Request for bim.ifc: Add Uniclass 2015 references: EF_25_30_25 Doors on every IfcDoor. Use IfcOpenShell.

First a look at what the model holds.

```python
import ifcopenshell

model = ifcopenshell.open("bim.ifc")
print(model.schema)
print("classifications:", [c.Name for c in model.by_type("IfcClassification")])
for ifc_class in ("IfcDoor", "IfcRoof", "IfcStair", "IfcWall", "IfcWindow"):
    print(ifc_class, len(model.by_type(ifc_class)))
```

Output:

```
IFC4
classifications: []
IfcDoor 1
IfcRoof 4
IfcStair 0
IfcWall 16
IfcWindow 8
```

```python
import ifcopenshell
import ifcopenshell.api.classification

model = ifcopenshell.open("bim.ifc")

system = ifcopenshell.api.classification.add_classification(model, classification="Uniclass 2015")

codes = {
    "IfcDoor": ("EF_25_30_25", "Doors"),
}
for ifc_class, (code, name) in codes.items():
    products = model.by_type(ifc_class)
    ifcopenshell.api.classification.add_reference(
        model, products=products, classification=system, identification=code, name=name
    )
    print(code, len(products))

model.write("bim_updated.ifc")
```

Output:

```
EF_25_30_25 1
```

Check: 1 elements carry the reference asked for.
